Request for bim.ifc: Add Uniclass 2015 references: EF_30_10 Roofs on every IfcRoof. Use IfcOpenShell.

First a look at what the model holds.

```python
import ifcopenshell

model = ifcopenshell.open("bim.ifc")
print(model.schema)
print("classifications:", [c.Name for c in model.by_type("IfcClassification")])
for ifc_class in ("IfcDoor", "IfcRoof", "IfcStair", "IfcWall", "IfcWindow"):
    print(ifc_class, len(model.by_type(ifc_class)))
```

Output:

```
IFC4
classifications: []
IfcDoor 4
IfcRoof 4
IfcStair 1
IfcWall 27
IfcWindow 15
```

```python
import ifcopenshell
import ifcopenshell.api.classification

model = ifcopenshell.open("bim.ifc")

system = ifcopenshell.api.classification.add_classification(model, classification="Uniclass 2015")

codes = {
    "IfcRoof": ("EF_30_10", "Roofs"),
}
for ifc_class, (code, name) in codes.items():
    products = model.by_type(ifc_class)
    ifcopenshell.api.classification.add_reference(
        model, products=products, classification=system, identification=code, name=name
    )
    print(code, len(products))

model.write("bim_updated.ifc")
```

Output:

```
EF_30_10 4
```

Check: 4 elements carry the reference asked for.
